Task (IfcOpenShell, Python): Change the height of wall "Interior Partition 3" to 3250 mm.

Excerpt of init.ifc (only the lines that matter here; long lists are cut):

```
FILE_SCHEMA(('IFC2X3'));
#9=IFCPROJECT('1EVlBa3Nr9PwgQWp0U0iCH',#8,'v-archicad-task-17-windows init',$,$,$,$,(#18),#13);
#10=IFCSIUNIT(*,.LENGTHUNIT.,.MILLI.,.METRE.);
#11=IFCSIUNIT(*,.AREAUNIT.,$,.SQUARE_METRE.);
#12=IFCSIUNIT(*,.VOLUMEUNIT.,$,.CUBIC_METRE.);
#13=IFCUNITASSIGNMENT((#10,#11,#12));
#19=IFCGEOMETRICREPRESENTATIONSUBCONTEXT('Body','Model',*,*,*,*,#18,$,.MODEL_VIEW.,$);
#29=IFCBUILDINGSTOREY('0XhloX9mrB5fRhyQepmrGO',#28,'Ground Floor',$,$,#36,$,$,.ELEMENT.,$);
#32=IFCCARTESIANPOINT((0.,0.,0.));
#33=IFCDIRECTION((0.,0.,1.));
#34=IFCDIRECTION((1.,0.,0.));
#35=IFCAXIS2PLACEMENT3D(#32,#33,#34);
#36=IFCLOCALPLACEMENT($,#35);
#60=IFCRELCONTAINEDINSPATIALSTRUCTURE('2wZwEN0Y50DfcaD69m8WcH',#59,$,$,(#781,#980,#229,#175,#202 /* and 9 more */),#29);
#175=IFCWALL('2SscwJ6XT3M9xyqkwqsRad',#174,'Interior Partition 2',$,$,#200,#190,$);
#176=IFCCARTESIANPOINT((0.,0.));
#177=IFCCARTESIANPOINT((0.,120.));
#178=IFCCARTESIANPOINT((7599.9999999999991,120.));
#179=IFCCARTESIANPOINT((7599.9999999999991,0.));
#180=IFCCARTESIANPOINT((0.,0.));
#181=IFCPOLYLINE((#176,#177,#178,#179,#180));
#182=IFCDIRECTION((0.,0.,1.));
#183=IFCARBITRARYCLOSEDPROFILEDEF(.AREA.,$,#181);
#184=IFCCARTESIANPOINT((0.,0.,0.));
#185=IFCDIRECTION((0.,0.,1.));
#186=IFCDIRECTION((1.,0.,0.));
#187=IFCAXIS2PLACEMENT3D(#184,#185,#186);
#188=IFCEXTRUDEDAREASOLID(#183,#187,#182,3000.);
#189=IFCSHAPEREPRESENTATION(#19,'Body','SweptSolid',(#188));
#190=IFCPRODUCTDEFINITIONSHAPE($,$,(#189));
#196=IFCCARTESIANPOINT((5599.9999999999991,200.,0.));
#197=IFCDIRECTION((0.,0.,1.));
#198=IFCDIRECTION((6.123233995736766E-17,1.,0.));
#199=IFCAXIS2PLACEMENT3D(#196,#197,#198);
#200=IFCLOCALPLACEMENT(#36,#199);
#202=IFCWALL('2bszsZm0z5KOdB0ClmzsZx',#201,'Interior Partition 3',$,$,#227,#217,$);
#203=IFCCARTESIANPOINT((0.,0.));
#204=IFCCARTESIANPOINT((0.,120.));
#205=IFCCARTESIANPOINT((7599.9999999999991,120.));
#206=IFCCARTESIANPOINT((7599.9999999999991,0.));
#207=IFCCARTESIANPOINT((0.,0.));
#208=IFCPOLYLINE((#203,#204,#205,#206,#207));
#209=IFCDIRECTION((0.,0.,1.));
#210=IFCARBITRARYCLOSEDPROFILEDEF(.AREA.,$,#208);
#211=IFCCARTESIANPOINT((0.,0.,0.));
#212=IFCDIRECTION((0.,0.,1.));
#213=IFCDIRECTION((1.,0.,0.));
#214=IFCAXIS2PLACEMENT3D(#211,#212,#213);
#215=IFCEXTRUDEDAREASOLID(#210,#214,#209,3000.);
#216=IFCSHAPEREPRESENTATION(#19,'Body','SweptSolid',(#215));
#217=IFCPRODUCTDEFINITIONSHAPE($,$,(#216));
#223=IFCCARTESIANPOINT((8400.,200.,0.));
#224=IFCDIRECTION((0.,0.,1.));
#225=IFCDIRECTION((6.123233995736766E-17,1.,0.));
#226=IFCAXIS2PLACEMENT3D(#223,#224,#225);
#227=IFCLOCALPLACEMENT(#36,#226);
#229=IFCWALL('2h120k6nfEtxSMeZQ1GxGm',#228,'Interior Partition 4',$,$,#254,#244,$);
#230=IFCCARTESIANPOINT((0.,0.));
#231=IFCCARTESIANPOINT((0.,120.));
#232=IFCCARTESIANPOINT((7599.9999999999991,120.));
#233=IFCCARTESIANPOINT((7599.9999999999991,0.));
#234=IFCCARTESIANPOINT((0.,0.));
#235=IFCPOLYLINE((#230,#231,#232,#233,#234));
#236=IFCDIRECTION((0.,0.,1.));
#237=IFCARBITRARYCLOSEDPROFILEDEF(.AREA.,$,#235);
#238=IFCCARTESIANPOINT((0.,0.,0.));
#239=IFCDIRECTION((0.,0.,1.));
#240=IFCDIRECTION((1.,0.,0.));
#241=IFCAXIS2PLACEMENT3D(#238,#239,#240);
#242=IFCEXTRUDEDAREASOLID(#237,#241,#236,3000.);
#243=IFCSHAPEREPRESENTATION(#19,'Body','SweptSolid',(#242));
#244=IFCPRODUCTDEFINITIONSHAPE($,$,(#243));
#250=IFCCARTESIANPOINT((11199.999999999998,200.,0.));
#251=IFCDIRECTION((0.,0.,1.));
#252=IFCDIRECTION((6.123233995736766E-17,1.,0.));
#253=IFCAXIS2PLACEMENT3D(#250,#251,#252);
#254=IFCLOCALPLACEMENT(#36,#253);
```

```python
import ifcopenshell
import ifcopenshell.geom
import ifcopenshell.util.representation
import ifcopenshell.util.shape
import ifcopenshell.util.unit

model = ifcopenshell.open("init.ifc")
unit_scale = ifcopenshell.util.unit.calculate_unit_scale(model)
settings = ifcopenshell.geom.settings()


def volume(element):
    """Net volume in cubic metres, openings subtracted."""
    shape = ifcopenshell.geom.create_shape(settings, element)
    return ifcopenshell.util.shape.get_volume(shape.geometry)


wall = model.by_id(202)
before = volume(wall)

body = ifcopenshell.util.representation.get_representation(wall, "Model", "Body")
solid = body.Items[0]
old_height = solid.Depth
solid.Depth = 3.25 / unit_scale
after = volume(wall)

print(f"height {old_height:g} -> {solid.Depth:g}, volume {before:.3f} -> {after:.3f} m3")

model.write("init_updated.ifc")
```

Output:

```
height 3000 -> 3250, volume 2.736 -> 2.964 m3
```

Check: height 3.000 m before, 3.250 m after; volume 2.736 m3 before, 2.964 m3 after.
